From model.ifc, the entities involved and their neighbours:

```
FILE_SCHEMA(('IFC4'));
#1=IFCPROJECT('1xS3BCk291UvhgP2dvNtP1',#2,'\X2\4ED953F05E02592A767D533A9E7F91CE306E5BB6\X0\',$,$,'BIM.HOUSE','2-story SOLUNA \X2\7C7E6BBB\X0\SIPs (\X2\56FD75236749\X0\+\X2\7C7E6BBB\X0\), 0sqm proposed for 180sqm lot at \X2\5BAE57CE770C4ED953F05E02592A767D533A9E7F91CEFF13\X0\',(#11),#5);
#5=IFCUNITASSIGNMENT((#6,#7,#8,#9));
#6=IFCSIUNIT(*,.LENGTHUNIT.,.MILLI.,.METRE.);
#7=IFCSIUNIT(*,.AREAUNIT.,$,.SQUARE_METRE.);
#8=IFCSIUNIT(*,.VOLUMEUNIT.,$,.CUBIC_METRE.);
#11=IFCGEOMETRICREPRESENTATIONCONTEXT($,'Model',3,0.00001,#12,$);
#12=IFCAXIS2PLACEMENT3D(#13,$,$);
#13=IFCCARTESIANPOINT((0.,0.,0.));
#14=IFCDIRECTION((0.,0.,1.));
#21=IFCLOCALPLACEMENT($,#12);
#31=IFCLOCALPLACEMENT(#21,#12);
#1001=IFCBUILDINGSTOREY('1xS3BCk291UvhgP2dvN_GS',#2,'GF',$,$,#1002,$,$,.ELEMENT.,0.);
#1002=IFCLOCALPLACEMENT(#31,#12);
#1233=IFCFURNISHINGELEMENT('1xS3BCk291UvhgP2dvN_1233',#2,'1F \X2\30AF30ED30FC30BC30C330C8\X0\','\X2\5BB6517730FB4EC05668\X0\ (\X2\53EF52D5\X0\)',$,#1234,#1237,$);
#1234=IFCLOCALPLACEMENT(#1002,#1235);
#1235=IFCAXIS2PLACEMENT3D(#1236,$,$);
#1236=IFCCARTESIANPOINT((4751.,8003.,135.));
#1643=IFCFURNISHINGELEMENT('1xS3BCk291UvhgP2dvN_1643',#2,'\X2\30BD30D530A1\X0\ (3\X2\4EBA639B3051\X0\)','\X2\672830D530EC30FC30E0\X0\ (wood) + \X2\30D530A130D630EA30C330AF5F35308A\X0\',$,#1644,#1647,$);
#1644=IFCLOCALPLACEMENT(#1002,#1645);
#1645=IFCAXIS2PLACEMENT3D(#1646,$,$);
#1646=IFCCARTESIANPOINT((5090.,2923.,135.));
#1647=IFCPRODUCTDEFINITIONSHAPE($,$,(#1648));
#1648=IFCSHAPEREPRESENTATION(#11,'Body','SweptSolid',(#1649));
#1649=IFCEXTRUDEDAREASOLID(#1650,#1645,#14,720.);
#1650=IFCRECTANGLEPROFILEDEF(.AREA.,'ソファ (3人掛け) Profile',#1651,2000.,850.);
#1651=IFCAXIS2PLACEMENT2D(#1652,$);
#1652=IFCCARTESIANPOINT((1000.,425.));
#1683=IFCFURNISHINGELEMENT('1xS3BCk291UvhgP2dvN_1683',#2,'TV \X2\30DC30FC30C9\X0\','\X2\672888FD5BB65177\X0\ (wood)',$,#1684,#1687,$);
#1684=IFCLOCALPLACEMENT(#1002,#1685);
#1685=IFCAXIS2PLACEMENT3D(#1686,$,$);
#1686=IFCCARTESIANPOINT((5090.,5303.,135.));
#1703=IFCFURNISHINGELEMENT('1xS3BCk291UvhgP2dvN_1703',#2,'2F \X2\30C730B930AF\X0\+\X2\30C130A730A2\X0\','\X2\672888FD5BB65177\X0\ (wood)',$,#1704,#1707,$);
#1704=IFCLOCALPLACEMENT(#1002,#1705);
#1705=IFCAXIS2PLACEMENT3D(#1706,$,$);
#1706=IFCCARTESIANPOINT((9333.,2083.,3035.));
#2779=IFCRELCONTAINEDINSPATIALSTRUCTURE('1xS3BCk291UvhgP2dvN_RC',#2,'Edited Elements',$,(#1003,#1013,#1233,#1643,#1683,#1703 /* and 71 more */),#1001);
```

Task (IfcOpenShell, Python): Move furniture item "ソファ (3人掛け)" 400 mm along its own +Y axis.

```python
import ifcopenshell
import ifcopenshell.api.geometry
import ifcopenshell.util.placement

model = ifcopenshell.open("model.ifc")

item = model.by_id(1643)
matrix = ifcopenshell.util.placement.get_local_placement(item.ObjectPlacement)
matrix[:3, 3] += matrix[:3, 1] * 400.0
ifcopenshell.api.geometry.edit_object_placement(model, product=item, matrix=matrix, is_si=False)

print(ifcopenshell.util.placement.get_local_placement(item.ObjectPlacement).round(3) + 0.0)

model.write("model_updated.ifc")
```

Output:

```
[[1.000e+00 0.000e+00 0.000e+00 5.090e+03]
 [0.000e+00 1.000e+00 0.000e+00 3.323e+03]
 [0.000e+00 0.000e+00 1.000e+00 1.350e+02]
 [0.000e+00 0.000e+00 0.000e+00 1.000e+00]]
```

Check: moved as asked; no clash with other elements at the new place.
